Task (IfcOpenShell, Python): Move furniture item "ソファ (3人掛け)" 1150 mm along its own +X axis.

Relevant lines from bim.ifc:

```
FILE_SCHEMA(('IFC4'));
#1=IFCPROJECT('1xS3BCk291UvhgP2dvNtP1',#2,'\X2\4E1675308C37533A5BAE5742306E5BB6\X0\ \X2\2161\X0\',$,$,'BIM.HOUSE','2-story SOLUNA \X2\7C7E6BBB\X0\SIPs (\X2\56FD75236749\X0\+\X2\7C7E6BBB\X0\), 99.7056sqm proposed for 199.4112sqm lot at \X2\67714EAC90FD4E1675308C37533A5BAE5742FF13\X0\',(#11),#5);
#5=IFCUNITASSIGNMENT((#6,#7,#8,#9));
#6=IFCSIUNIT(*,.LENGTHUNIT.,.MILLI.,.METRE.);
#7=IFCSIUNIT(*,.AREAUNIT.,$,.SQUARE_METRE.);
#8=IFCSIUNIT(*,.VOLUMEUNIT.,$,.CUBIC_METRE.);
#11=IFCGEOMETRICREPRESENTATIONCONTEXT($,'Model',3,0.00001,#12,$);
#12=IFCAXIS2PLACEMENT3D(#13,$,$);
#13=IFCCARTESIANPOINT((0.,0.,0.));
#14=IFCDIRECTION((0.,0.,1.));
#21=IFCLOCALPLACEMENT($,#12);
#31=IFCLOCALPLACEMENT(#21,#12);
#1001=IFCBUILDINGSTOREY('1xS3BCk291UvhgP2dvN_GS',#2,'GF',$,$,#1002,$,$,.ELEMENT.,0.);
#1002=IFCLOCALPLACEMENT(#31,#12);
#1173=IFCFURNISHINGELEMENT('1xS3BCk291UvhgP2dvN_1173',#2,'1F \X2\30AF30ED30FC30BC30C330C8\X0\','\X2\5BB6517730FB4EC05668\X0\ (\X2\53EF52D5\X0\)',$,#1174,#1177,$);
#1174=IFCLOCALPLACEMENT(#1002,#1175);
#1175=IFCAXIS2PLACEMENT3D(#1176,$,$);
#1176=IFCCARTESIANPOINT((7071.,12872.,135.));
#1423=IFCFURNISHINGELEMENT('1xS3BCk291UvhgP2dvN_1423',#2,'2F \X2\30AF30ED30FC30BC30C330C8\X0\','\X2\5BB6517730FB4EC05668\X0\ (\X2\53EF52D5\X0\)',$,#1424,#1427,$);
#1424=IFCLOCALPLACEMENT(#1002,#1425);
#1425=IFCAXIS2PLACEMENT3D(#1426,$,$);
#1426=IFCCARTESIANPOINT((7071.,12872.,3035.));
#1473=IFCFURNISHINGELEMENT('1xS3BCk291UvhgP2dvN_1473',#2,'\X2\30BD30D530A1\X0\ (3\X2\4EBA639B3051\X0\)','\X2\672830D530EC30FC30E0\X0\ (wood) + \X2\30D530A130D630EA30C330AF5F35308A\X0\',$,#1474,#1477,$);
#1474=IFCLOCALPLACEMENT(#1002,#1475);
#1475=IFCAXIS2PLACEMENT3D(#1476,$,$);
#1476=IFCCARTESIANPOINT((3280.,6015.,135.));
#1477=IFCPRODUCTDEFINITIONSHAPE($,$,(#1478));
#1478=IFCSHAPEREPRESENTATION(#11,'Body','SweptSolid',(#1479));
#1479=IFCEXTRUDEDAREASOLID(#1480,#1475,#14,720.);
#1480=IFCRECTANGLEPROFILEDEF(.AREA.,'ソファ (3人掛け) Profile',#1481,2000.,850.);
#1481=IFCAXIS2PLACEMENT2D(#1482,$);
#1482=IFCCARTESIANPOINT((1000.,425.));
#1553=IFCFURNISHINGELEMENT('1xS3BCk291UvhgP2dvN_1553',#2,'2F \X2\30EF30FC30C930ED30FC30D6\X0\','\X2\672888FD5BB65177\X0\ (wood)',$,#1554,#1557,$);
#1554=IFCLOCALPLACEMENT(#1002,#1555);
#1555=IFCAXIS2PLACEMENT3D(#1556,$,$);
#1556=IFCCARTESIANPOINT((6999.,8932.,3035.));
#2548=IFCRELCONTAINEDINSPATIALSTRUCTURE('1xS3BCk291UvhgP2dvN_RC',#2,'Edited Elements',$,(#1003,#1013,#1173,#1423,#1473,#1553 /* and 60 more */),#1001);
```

```python
import ifcopenshell
import ifcopenshell.api.geometry
import ifcopenshell.util.placement
import ifcopenshell.util.unit

model = ifcopenshell.open("bim.ifc")
unit_scale = ifcopenshell.util.unit.calculate_unit_scale(model)

item = model.by_guid("1xS3BCk291UvhgP2dvN_1473")
matrix = ifcopenshell.util.placement.get_local_placement(item.ObjectPlacement)
matrix[:3, 3] += matrix[:3, 0] * 1.15 / unit_scale
ifcopenshell.api.geometry.edit_object_placement(model, product=item, matrix=matrix, is_si=False)

print(ifcopenshell.util.placement.get_local_placement(item.ObjectPlacement).round(3) + 0.0)

model.write("bim_rev.ifc")
```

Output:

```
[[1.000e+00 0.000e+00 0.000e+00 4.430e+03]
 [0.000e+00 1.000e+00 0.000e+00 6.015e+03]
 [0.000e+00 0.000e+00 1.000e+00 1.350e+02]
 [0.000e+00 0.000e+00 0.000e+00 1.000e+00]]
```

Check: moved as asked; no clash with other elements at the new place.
